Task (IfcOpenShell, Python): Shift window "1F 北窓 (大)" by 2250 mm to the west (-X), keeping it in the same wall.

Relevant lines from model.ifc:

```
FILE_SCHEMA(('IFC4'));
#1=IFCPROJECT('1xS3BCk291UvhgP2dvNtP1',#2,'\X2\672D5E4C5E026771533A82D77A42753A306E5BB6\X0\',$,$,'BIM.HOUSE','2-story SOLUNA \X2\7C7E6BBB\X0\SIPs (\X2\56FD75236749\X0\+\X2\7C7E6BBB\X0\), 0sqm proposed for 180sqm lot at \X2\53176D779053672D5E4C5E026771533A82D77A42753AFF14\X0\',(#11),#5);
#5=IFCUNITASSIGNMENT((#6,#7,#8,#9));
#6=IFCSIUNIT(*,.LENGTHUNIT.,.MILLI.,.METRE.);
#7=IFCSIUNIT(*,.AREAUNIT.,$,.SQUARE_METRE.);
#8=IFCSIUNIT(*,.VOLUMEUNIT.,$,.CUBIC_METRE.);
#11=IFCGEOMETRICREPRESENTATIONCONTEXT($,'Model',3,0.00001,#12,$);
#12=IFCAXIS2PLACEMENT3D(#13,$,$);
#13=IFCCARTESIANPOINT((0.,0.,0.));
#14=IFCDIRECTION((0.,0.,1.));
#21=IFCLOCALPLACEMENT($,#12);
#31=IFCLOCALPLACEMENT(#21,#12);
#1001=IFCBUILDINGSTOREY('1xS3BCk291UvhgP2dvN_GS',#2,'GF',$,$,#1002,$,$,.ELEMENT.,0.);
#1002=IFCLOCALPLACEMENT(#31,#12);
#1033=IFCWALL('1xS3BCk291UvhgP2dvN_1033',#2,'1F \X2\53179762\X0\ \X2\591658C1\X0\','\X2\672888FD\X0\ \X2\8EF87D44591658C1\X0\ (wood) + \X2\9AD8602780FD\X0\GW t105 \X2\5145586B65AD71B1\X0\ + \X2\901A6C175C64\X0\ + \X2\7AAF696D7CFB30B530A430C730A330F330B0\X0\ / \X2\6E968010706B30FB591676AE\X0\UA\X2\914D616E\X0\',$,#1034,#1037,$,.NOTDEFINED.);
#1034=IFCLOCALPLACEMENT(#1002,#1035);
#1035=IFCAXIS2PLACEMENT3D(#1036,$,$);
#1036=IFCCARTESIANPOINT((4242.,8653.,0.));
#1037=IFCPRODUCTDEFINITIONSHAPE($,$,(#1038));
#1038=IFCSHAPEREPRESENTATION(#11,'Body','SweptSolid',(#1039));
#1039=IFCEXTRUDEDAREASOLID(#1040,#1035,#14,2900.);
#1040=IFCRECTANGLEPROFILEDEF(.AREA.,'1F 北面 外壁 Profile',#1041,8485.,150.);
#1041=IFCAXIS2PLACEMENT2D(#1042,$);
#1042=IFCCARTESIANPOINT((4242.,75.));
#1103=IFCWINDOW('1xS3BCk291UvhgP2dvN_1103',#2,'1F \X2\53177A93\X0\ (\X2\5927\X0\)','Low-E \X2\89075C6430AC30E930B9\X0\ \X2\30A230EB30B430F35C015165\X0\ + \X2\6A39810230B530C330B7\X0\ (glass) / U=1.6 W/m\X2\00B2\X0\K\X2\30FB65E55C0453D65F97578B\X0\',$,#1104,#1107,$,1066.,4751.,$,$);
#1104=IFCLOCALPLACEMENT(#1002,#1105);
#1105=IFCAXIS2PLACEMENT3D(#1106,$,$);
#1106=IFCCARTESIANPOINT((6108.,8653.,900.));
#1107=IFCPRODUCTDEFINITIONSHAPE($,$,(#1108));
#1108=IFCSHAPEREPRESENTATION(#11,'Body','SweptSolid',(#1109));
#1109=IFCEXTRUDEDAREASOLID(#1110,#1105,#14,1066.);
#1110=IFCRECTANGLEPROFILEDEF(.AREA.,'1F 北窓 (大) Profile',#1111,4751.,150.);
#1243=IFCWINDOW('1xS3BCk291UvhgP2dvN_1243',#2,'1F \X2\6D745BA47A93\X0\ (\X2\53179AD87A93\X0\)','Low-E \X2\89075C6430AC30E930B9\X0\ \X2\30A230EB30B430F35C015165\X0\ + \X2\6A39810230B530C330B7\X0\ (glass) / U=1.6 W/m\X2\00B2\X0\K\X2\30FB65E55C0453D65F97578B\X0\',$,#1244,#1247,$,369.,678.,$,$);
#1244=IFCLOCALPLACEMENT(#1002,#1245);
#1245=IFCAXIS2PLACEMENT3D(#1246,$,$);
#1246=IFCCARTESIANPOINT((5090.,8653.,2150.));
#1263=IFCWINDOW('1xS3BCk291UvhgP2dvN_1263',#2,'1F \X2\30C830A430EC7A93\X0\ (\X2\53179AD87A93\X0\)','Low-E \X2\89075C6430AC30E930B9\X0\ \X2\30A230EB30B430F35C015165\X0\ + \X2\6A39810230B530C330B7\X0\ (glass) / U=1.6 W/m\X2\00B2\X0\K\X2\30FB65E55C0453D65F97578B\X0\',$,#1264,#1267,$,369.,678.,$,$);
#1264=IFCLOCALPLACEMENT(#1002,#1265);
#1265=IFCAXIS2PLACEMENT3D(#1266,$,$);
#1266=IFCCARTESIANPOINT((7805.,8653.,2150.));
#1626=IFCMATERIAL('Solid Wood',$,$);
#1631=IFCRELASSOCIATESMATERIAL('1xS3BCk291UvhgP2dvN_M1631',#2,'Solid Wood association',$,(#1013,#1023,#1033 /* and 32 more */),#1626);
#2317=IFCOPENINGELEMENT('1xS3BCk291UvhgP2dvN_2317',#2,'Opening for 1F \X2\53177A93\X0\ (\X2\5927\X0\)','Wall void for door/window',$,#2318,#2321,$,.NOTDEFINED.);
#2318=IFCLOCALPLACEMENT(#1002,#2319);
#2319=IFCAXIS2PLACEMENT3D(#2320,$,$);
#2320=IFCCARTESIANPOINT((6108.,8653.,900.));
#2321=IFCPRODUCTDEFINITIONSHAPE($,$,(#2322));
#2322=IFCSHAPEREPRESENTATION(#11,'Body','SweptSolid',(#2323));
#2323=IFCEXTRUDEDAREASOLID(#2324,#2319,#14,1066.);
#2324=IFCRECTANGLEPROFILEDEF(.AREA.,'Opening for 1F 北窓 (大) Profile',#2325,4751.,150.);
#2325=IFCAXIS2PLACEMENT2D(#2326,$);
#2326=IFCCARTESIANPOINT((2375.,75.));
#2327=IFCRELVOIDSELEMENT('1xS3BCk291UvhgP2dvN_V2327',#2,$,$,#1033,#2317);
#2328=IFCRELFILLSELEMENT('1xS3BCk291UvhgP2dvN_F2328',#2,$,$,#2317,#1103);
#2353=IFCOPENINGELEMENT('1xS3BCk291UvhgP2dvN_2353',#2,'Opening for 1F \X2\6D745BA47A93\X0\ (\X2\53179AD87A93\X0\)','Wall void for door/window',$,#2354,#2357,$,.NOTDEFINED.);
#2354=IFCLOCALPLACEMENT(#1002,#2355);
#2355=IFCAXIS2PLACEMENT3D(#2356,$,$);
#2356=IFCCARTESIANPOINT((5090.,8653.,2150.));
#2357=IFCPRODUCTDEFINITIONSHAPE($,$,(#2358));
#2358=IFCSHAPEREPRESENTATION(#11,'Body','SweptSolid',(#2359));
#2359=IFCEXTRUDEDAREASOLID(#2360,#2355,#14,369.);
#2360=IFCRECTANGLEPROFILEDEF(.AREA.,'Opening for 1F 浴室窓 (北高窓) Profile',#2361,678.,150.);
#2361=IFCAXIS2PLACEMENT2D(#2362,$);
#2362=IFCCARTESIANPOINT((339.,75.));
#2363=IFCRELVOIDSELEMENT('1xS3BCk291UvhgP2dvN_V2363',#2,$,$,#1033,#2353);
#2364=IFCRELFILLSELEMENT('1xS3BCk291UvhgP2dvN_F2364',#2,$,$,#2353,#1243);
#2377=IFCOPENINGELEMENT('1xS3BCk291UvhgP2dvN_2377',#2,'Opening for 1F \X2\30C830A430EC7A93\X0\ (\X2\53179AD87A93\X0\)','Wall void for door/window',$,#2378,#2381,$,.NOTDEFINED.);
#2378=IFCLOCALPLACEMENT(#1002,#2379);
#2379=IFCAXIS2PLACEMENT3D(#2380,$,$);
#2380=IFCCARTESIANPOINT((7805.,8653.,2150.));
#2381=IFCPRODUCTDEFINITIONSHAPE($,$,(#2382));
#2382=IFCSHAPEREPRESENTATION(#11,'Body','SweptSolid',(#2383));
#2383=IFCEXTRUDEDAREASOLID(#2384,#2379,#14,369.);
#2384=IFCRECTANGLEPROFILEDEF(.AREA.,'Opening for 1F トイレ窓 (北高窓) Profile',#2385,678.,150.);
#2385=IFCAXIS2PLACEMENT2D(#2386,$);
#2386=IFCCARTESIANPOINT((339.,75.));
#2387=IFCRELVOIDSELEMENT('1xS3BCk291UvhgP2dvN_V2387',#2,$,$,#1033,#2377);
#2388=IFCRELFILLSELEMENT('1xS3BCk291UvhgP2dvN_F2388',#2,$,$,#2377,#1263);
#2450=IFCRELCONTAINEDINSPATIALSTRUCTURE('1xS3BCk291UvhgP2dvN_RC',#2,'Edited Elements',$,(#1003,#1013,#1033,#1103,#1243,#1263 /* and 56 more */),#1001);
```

```python
import ifcopenshell
import ifcopenshell.api.geometry
import ifcopenshell.util.placement
import ifcopenshell.util.unit

model = ifcopenshell.open("model.ifc")
unit_scale = ifcopenshell.util.unit.calculate_unit_scale(model)

window = model.by_guid("1xS3BCk291UvhgP2dvN_1103")
opening = window.FillsVoids[0].RelatingOpeningElement
wall = opening.VoidsElements[0].RelatingBuildingElement

wall_matrix = ifcopenshell.util.placement.get_local_placement(wall.ObjectPlacement)
shift = wall_matrix[:3, 0] * -2.25 / unit_scale
before = ifcopenshell.util.placement.get_local_placement(window.ObjectPlacement)[:3, 3].copy()

# The window is not placed relative to its opening, so move both.
for product in (opening, window):
    matrix = ifcopenshell.util.placement.get_local_placement(product.ObjectPlacement)
    matrix[:3, 3] += shift
    ifcopenshell.api.geometry.edit_object_placement(model, product=product, matrix=matrix, is_si=False)

after = ifcopenshell.util.placement.get_local_placement(window.ObjectPlacement)[:3, 3]
print("window moved by", (after - before).round(3) + 0.0)

model.write("model_rev.ifc")
```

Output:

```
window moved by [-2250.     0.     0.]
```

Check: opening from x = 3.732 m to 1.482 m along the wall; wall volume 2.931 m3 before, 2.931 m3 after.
